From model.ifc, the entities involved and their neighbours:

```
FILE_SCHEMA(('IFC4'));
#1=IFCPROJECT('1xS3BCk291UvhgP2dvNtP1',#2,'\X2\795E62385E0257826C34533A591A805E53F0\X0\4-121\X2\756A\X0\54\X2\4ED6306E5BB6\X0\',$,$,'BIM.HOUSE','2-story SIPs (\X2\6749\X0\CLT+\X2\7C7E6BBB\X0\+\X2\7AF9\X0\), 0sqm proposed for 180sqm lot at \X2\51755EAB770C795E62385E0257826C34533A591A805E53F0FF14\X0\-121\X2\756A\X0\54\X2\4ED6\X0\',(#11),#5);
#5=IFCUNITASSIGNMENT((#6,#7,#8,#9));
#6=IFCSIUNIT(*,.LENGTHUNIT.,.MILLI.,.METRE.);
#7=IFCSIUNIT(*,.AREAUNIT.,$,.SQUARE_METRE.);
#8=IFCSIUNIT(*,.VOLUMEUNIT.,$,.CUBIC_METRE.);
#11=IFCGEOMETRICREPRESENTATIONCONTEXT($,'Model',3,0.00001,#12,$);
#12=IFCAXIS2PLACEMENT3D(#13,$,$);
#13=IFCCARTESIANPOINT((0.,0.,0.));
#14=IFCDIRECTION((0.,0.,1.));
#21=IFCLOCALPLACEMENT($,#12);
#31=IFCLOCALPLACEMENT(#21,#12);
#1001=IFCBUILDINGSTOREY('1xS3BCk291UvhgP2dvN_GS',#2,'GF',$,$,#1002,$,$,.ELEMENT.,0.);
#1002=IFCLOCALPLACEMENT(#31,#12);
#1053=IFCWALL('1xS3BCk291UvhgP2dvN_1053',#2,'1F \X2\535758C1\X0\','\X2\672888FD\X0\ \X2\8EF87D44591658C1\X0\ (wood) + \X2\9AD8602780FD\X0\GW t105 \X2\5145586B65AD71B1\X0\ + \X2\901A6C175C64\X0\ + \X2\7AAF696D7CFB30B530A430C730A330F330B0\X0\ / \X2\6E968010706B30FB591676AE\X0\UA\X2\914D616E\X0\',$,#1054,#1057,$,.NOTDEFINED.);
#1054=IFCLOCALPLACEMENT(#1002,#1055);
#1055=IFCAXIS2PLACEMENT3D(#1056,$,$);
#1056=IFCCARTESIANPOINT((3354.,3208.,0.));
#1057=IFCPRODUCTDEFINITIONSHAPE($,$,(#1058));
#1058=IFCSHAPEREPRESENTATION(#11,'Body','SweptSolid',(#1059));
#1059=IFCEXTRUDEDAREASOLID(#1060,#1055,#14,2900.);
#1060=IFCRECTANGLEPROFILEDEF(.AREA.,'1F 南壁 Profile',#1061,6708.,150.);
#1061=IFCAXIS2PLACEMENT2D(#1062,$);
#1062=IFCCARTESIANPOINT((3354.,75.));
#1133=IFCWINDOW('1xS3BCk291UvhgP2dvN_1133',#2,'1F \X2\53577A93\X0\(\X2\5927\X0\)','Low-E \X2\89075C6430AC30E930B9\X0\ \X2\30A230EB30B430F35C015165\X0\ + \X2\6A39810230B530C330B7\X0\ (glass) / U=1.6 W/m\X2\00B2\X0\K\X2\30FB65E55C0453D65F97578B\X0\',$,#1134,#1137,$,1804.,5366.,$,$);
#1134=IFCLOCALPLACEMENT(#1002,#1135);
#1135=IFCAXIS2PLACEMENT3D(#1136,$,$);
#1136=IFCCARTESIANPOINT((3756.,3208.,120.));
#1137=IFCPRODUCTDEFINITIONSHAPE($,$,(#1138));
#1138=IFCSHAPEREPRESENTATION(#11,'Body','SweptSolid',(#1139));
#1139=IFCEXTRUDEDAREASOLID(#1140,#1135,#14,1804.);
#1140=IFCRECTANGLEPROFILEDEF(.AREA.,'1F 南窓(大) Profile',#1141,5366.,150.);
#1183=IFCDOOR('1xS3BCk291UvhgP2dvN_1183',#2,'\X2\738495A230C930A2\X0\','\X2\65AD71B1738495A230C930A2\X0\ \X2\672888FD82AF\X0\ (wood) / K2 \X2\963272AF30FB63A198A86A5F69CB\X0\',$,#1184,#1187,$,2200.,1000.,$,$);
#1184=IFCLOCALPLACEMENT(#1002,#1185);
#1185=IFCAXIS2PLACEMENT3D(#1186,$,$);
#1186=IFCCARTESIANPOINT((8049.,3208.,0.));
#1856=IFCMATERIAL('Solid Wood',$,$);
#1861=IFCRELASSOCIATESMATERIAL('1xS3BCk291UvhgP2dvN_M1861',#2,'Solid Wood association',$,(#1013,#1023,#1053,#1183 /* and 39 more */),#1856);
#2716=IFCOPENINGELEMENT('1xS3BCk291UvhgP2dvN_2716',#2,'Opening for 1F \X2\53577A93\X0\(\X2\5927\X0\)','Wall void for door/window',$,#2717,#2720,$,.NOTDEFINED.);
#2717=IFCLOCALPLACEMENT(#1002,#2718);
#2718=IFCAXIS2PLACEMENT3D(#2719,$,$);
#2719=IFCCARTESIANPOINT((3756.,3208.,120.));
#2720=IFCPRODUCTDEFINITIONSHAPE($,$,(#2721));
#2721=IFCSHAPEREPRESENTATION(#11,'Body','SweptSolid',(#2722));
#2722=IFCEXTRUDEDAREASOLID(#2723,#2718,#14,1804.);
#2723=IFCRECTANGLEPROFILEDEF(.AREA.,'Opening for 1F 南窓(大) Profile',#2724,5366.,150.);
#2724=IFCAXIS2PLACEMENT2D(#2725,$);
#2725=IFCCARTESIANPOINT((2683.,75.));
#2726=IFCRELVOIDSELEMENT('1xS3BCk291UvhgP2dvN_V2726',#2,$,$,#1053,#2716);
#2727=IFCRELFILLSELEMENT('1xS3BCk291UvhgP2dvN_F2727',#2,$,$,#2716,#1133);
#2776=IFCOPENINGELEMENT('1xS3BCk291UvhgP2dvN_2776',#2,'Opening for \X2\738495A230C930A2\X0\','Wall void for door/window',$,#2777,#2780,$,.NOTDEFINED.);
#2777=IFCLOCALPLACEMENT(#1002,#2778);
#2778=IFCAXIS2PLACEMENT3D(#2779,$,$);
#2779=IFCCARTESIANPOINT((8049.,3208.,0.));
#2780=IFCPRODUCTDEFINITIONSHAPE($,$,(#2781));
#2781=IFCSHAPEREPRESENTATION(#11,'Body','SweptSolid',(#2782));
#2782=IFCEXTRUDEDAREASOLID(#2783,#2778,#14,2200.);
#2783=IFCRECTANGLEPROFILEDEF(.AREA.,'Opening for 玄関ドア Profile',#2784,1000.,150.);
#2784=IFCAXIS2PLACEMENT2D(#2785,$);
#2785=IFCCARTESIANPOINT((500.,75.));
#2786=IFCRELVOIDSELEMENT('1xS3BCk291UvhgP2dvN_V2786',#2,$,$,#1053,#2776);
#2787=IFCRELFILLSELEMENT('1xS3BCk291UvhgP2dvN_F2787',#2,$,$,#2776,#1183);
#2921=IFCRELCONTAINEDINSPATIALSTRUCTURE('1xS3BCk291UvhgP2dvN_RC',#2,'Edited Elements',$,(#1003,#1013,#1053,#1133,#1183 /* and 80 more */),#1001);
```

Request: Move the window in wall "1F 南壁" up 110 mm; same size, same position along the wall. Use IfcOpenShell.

```python
import numpy as np
import ifcopenshell
import ifcopenshell.api.geometry
import ifcopenshell.util.placement
import ifcopenshell.util.unit

model = ifcopenshell.open("model.ifc")
unit_scale = ifcopenshell.util.unit.calculate_unit_scale(model)

window = model.by_id(1133)
opening = window.FillsVoids[0].RelatingOpeningElement
dz = 0.11 / unit_scale

shift = np.array([0.0, 0.0, dz])
# The window is not placed relative to its opening, so move both.
for product in (opening, window):
    matrix = ifcopenshell.util.placement.get_local_placement(product.ObjectPlacement)
    matrix[:3, 3] += shift
    ifcopenshell.api.geometry.edit_object_placement(model, product=product, matrix=matrix, is_si=False)

print(f"moved by {dz * unit_scale:+.3f} m")

model.write("model_v2.ifc")
```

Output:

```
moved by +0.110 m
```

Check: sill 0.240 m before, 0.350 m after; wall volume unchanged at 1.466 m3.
